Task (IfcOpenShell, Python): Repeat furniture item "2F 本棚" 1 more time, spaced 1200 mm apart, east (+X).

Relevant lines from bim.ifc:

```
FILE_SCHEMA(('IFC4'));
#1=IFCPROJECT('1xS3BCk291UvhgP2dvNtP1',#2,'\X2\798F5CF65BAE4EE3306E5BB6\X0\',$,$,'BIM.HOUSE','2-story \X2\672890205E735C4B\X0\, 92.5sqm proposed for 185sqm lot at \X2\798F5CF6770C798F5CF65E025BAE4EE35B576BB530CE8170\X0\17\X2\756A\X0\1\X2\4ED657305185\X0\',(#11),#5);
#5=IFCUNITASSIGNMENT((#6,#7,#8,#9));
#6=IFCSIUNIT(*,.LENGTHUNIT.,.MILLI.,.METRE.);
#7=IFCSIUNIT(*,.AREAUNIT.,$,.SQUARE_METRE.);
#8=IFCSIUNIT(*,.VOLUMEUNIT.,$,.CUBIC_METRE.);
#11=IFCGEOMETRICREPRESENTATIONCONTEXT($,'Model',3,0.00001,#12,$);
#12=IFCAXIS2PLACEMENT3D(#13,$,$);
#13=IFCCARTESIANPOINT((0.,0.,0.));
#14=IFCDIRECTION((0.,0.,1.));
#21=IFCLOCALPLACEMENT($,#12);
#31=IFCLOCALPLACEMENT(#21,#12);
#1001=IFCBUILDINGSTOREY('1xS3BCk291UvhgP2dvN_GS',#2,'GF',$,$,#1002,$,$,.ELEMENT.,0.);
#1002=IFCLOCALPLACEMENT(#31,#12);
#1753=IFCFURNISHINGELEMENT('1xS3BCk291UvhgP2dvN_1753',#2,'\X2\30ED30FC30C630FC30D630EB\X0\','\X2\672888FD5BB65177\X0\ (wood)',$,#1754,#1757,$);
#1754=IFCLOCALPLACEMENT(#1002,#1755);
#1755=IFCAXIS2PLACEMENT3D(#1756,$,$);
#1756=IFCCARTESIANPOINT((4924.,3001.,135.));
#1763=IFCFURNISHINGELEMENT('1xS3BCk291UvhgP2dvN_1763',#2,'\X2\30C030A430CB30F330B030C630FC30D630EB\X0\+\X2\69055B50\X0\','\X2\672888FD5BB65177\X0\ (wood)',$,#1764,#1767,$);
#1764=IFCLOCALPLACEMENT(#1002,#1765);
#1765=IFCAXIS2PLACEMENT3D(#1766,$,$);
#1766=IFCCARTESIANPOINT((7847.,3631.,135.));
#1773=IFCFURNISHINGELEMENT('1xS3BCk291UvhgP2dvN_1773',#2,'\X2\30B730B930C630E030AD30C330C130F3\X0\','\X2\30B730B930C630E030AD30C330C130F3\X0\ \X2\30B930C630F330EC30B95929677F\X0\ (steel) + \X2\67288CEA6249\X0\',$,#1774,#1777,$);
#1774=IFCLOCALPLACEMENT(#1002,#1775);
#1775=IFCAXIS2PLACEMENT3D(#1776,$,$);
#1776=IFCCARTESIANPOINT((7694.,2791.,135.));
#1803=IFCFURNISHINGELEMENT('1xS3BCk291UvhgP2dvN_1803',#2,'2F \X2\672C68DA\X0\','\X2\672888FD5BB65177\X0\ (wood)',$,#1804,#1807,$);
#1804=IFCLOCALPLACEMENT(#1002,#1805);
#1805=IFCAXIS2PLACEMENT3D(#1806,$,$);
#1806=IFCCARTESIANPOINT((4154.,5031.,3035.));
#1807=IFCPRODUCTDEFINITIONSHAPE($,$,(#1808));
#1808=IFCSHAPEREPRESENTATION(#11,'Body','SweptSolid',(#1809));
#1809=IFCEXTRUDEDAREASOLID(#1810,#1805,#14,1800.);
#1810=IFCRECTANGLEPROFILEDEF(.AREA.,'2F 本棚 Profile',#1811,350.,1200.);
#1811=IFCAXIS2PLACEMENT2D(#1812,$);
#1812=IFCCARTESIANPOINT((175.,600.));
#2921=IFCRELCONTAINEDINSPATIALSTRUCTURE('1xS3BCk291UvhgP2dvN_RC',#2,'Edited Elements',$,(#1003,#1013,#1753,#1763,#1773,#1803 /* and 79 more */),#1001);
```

```python
import numpy as np
import ifcopenshell
import ifcopenshell.api.geometry
import ifcopenshell.api.root
import ifcopenshell.util.element
import ifcopenshell.util.placement
import ifcopenshell.util.unit

model = ifcopenshell.open("bim.ifc")
unit_scale = ifcopenshell.util.unit.calculate_unit_scale(model)


def reuse_history(source, copy):
    """copy_class also copies each property set's owner history, people and application; keep the originals."""
    for rel in copy.IsDefinedBy:
        if rel.is_a("IfcRelDefinesByProperties") and (history := rel.RelatingPropertyDefinition.OwnerHistory):
            rel.RelatingPropertyDefinition.OwnerHistory = source.OwnerHistory
            ifcopenshell.util.element.remove_deep2(model, history)


source = model.by_id(1803)
base = ifcopenshell.util.placement.get_local_placement(source.ObjectPlacement)
step = np.array([1.0, 0.0, 0.0]) * 1.2 / unit_scale

for i in range(1, 2):
    copy = ifcopenshell.api.root.copy_class(model, product=source)
    copy.Representation = ifcopenshell.util.element.copy_deep(
        model, source.Representation, exclude=["IfcGeometricRepresentationContext", "IfcRepresentationMap"]
    )
    reuse_history(source, copy)
    matrix = base.copy()
    matrix[:3, 3] += i * step
    print("added at", matrix[:3, 3].round(3) + 0.0)
    ifcopenshell.api.geometry.edit_object_placement(model, product=copy, matrix=matrix, is_si=False)

model.write("bim_edited.ifc")
```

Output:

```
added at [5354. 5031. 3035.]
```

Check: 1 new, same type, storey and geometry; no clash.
